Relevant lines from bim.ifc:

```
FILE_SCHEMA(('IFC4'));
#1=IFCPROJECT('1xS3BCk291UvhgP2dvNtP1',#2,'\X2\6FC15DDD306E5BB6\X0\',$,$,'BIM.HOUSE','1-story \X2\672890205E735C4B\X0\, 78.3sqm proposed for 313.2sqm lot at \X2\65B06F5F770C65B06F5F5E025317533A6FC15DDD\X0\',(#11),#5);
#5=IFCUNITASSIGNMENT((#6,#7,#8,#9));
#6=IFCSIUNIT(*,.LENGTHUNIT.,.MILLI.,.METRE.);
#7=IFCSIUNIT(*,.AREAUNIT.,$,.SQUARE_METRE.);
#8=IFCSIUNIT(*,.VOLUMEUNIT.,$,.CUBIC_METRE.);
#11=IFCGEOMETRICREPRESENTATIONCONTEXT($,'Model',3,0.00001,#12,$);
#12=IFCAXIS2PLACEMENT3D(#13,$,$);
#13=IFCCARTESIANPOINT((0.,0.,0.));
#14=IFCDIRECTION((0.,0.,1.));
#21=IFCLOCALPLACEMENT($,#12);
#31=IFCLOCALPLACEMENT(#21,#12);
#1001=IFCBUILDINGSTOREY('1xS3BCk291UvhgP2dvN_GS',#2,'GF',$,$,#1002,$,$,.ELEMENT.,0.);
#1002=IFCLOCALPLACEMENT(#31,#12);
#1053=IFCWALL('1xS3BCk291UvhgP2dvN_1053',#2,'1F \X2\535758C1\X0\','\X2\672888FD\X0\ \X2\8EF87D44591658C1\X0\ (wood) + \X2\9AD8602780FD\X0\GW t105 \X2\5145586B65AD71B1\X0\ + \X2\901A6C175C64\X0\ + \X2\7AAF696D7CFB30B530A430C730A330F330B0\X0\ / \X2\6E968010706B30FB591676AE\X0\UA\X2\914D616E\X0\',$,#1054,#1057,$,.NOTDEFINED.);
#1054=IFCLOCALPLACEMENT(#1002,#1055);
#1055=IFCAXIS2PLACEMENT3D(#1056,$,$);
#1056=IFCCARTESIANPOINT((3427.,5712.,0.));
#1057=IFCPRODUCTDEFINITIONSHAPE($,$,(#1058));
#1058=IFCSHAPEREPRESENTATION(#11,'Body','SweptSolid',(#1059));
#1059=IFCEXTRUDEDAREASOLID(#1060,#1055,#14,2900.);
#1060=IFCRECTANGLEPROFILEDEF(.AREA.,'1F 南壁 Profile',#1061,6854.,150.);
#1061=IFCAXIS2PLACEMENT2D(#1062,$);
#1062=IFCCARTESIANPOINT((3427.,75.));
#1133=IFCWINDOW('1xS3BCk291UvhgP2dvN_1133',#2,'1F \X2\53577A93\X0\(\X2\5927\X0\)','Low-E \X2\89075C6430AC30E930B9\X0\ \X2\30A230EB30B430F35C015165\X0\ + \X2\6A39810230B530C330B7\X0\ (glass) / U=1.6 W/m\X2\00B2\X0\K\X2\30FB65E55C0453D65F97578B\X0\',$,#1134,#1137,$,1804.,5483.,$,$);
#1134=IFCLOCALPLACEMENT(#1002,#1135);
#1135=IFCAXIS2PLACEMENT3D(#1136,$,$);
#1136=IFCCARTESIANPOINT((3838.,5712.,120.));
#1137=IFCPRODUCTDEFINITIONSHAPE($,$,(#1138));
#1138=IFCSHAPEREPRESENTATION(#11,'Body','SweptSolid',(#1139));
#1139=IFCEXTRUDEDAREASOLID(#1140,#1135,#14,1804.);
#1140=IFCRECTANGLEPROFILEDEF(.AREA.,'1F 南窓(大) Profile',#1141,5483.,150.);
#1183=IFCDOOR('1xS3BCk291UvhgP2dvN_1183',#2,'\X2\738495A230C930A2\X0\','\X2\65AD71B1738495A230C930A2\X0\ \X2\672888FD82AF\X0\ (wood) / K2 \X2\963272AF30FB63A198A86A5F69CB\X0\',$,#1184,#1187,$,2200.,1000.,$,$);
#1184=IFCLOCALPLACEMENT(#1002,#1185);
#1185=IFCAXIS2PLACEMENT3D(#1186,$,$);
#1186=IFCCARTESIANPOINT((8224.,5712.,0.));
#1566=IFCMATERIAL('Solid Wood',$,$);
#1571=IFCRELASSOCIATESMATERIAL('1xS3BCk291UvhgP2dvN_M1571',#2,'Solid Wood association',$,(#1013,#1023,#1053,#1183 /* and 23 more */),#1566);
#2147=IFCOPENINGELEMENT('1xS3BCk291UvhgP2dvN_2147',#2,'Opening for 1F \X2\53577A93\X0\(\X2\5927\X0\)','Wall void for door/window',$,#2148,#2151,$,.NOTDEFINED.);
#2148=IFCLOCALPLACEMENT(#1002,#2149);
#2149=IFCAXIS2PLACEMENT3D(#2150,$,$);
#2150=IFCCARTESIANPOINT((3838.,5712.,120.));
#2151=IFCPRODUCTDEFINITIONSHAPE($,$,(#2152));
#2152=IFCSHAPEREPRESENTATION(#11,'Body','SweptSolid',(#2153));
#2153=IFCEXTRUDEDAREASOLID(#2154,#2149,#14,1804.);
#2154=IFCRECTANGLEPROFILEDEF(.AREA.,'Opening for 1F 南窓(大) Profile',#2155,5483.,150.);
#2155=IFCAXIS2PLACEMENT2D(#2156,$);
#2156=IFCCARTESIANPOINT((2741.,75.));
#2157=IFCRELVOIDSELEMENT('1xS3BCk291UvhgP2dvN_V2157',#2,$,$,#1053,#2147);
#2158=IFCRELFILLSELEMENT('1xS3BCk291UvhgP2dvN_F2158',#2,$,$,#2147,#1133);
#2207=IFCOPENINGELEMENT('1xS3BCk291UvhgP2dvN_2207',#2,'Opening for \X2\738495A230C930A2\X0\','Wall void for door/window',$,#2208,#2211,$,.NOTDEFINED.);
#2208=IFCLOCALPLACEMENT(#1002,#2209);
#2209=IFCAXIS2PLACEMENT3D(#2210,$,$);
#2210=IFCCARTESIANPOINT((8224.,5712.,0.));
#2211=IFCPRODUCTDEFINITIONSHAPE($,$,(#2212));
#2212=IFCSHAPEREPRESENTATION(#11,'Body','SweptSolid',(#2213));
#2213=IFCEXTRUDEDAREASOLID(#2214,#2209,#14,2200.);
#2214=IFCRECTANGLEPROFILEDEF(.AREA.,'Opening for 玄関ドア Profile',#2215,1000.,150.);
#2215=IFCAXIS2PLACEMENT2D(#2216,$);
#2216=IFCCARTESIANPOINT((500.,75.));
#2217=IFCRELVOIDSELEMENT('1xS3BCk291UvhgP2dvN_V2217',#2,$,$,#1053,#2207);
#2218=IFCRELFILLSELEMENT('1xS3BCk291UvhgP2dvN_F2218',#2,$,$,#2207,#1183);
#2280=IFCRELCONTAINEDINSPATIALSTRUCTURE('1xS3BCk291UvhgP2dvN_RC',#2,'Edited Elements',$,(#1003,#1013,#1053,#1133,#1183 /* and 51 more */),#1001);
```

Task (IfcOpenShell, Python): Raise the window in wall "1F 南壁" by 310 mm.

```python
import numpy as np
import ifcopenshell
import ifcopenshell.api.geometry
import ifcopenshell.util.placement
import ifcopenshell.util.unit

model = ifcopenshell.open("bim.ifc")
unit_scale = ifcopenshell.util.unit.calculate_unit_scale(model)

window = model.by_id(1133)
opening = window.FillsVoids[0].RelatingOpeningElement
dz = 0.31 / unit_scale

shift = np.array([0.0, 0.0, dz])
# The window is not placed relative to its opening, so move both.
for product in (opening, window):
    matrix = ifcopenshell.util.placement.get_local_placement(product.ObjectPlacement)
    matrix[:3, 3] += shift
    ifcopenshell.api.geometry.edit_object_placement(model, product=product, matrix=matrix, is_si=False)

print(f"moved by {dz * unit_scale:+.3f} m")

model.write("bim_rev.ifc")
```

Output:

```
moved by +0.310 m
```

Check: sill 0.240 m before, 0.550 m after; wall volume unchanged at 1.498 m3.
